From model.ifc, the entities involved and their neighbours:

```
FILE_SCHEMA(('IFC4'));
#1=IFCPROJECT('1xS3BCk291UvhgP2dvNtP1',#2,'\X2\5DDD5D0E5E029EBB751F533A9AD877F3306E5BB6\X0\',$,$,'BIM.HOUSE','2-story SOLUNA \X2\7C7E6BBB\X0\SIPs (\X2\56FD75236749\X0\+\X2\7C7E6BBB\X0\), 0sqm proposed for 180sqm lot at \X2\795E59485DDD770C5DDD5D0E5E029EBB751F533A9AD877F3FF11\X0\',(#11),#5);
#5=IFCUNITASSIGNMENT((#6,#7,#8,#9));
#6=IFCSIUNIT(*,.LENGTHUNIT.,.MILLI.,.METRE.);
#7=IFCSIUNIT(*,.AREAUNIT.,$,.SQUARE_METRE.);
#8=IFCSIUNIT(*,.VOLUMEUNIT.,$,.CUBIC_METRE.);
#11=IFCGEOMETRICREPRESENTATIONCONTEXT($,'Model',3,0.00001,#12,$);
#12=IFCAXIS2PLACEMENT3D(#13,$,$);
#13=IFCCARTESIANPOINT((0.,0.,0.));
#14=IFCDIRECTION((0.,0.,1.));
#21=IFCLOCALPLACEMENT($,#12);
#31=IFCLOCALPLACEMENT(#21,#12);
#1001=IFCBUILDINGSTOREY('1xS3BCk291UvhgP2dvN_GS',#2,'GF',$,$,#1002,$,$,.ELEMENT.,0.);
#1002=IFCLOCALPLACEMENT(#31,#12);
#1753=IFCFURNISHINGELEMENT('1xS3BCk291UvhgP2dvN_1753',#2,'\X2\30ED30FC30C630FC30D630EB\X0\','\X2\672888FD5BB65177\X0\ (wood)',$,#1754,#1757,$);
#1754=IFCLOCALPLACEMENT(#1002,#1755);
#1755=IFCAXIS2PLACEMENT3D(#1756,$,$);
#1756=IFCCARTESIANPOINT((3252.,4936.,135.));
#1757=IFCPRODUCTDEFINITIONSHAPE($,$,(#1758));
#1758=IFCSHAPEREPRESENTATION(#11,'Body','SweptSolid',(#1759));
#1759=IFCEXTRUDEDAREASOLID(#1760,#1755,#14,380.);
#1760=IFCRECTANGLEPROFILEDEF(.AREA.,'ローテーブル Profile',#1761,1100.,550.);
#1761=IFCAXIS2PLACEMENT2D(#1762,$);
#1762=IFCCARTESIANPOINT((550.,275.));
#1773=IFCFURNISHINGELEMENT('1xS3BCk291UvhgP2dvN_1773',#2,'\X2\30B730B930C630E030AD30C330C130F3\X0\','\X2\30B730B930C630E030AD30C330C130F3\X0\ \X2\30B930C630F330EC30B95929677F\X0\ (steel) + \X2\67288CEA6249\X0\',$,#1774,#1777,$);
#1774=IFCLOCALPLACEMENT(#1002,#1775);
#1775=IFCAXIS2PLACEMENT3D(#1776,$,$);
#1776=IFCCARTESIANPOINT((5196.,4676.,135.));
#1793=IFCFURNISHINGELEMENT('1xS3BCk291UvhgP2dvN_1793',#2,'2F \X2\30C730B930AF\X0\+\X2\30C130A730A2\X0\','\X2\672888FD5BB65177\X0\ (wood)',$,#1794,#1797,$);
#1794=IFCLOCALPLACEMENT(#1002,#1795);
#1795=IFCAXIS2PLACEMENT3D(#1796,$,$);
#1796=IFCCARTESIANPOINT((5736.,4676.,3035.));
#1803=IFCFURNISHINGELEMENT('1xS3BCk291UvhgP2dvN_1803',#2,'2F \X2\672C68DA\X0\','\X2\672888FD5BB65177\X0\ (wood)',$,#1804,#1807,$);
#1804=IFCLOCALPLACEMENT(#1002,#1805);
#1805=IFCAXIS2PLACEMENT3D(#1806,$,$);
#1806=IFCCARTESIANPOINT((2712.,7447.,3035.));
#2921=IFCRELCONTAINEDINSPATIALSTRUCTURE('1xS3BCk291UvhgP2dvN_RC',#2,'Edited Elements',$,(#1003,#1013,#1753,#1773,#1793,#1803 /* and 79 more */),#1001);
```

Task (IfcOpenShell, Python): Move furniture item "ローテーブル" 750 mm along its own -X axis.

```python
import ifcopenshell
import ifcopenshell.api.geometry
import ifcopenshell.util.placement
import ifcopenshell.util.unit

model = ifcopenshell.open("model.ifc")
unit_scale = ifcopenshell.util.unit.calculate_unit_scale(model)

item = model.by_id(1753)
matrix = ifcopenshell.util.placement.get_local_placement(item.ObjectPlacement)
matrix[:3, 3] -= matrix[:3, 0] * 0.75 / unit_scale
ifcopenshell.api.geometry.edit_object_placement(model, product=item, matrix=matrix, is_si=False)

print(ifcopenshell.util.placement.get_local_placement(item.ObjectPlacement).round(3) + 0.0)

model.write("model_rev.ifc")
```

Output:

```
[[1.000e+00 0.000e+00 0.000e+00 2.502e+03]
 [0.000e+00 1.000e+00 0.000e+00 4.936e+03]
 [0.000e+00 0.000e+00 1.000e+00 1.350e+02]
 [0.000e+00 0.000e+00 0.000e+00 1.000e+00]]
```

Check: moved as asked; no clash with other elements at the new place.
